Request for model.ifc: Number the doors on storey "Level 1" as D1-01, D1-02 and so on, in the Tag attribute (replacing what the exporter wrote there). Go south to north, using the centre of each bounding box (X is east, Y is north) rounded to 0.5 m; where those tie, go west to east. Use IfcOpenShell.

First a look at what the model holds.

```python
import ifcopenshell
import ifcopenshell.util.element
import ifcopenshell.util.placement

model = ifcopenshell.open("model.ifc")
print(model.schema)
storey = next(s for s in model.by_type("IfcBuildingStorey") if s.Name == "Level 1")
doors = [e for e in ifcopenshell.util.element.get_decomposition(storey) if e.is_a("IfcDoor")]
for e in sorted(doors, key=lambda e: e.id()):
    origin = ifcopenshell.util.placement.get_local_placement(e.ObjectPlacement)[:3, 3]
    print(e.id(), e.Tag, e.Name, origin.round(2) + 0.0, sep=" | ")
```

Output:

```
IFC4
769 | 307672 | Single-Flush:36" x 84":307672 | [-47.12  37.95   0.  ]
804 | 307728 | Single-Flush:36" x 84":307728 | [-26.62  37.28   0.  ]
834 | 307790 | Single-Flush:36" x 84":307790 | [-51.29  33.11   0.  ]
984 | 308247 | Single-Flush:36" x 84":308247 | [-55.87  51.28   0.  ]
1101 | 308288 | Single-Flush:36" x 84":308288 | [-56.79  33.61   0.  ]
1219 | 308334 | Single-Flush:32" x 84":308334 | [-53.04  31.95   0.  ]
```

```python
import ifcopenshell
import ifcopenshell.geom
import ifcopenshell.util.element
import ifcopenshell.util.shape

model = ifcopenshell.open("model.ifc")
settings = ifcopenshell.geom.settings()
settings.set("use-world-coords", True)


def centre(element):
    shape = ifcopenshell.geom.create_shape(settings, element)
    return ifcopenshell.util.shape.get_bbox_centroid(shape.geometry)


storey = next(s for s in model.by_type("IfcBuildingStorey") if s.Name == "Level 1")
doors = [e for e in ifcopenshell.util.element.get_decomposition(storey) if e.is_a("IfcDoor")]

# Insertion points can sit at a corner or the storey origin, so sort by the geometry (in metres).
centres = {e: centre(e) for e in doors}
doors.sort(key=lambda e: (round(centres[e][1] / 0.5), centres[e][0]))

for i, e in enumerate(doors, start=1):
    number = f"D1-{i:02d}"
    e.Tag = number
    print(e.id(), number)

model.write("model_edited.ifc")
```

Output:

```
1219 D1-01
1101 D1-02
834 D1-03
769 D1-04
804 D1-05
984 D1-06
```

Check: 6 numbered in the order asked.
